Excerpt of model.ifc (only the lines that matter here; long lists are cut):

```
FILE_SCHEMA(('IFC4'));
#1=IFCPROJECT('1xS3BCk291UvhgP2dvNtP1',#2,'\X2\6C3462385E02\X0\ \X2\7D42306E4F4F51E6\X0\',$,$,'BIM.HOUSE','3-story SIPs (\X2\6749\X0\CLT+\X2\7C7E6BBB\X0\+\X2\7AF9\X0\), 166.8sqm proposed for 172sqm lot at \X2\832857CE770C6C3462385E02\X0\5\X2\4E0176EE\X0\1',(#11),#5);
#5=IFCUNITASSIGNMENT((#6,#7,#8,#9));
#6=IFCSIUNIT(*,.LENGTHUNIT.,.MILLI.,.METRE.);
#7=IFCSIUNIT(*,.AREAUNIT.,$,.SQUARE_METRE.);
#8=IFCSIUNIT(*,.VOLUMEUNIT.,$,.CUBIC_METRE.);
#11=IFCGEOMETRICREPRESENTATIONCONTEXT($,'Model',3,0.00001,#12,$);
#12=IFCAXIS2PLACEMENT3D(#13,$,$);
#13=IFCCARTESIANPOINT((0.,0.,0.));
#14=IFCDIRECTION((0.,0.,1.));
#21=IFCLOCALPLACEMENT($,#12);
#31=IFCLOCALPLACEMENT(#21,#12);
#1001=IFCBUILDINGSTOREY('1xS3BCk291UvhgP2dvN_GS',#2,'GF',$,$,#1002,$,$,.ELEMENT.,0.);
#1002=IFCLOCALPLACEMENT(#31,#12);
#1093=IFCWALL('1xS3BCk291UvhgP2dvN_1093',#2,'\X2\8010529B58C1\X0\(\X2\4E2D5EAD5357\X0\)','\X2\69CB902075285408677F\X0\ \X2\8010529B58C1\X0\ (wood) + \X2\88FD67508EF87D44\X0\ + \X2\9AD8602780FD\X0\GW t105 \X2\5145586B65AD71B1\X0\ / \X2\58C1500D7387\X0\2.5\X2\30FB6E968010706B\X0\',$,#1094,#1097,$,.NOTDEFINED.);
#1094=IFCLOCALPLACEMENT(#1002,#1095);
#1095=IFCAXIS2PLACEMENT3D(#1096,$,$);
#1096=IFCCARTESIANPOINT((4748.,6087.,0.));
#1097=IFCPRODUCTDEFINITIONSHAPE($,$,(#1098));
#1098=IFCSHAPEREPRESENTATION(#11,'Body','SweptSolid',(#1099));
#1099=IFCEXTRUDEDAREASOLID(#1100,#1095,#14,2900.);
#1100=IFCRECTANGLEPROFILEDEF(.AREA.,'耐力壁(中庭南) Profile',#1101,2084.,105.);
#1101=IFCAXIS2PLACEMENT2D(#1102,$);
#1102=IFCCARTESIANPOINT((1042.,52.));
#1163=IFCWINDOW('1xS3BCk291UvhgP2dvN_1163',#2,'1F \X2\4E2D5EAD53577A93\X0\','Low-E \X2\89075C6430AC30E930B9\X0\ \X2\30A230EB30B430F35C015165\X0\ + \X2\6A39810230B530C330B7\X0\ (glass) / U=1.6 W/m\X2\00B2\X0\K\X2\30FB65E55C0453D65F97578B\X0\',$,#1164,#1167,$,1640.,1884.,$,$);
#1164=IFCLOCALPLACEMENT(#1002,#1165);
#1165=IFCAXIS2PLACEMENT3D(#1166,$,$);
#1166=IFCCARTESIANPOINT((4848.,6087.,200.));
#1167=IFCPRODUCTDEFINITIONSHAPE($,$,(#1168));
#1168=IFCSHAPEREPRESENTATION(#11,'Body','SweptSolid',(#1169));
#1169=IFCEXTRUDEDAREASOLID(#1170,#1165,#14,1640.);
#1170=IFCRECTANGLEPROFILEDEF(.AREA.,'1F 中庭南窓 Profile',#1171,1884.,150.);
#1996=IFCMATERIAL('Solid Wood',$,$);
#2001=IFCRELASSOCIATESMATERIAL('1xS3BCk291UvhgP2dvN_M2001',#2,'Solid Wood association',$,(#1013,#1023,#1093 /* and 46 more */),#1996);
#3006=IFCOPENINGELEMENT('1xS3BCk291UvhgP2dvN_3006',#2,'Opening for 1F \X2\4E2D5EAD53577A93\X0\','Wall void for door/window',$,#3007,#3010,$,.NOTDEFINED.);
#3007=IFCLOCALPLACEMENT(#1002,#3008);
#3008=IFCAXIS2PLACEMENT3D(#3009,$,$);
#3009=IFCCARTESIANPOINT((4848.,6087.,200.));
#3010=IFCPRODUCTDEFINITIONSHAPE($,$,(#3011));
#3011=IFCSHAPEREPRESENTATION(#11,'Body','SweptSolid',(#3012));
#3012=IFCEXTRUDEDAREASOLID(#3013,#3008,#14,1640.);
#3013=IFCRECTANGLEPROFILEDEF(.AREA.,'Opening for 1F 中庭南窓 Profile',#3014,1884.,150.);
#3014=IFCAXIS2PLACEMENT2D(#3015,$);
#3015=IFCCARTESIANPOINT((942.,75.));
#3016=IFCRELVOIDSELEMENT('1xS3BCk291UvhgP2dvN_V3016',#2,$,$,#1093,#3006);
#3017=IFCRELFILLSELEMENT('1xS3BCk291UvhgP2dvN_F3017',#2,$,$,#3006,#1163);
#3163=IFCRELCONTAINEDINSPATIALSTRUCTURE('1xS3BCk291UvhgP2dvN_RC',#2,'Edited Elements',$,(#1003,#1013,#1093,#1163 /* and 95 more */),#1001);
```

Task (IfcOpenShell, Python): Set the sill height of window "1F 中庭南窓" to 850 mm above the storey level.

```python
import numpy as np
import ifcopenshell
import ifcopenshell.api.geometry
import ifcopenshell.geom
import ifcopenshell.util.element
import ifcopenshell.util.placement
import ifcopenshell.util.shape
import ifcopenshell.util.unit

model = ifcopenshell.open("model.ifc")
unit_scale = ifcopenshell.util.unit.calculate_unit_scale(model)

window = model.by_id(1163)
opening = window.FillsVoids[0].RelatingOpeningElement
storey = ifcopenshell.util.element.get_container(window, ifc_class="IfcBuildingStorey")
level = ifcopenshell.util.placement.get_local_placement(storey.ObjectPlacement)[2, 3]

# The opening's origin need not be at the sill, so measure its lowest point.
shape = ifcopenshell.geom.create_shape(ifcopenshell.geom.settings(), opening)
bottom = ifcopenshell.util.shape.get_shape_bottom_elevation(shape, shape.geometry) / unit_scale
dz = level + 0.85 / unit_scale - bottom

shift = np.array([0.0, 0.0, dz])
# The window is not placed relative to its opening, so move both.
for product in (opening, window):
    matrix = ifcopenshell.util.placement.get_local_placement(product.ObjectPlacement)
    matrix[:3, 3] += shift
    ifcopenshell.api.geometry.edit_object_placement(model, product=product, matrix=matrix, is_si=False)

print(f"moved by {dz * unit_scale:+.3f} m")

model.write("model_v2.ifc")
```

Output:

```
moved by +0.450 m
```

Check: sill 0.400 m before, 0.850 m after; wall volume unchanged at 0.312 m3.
